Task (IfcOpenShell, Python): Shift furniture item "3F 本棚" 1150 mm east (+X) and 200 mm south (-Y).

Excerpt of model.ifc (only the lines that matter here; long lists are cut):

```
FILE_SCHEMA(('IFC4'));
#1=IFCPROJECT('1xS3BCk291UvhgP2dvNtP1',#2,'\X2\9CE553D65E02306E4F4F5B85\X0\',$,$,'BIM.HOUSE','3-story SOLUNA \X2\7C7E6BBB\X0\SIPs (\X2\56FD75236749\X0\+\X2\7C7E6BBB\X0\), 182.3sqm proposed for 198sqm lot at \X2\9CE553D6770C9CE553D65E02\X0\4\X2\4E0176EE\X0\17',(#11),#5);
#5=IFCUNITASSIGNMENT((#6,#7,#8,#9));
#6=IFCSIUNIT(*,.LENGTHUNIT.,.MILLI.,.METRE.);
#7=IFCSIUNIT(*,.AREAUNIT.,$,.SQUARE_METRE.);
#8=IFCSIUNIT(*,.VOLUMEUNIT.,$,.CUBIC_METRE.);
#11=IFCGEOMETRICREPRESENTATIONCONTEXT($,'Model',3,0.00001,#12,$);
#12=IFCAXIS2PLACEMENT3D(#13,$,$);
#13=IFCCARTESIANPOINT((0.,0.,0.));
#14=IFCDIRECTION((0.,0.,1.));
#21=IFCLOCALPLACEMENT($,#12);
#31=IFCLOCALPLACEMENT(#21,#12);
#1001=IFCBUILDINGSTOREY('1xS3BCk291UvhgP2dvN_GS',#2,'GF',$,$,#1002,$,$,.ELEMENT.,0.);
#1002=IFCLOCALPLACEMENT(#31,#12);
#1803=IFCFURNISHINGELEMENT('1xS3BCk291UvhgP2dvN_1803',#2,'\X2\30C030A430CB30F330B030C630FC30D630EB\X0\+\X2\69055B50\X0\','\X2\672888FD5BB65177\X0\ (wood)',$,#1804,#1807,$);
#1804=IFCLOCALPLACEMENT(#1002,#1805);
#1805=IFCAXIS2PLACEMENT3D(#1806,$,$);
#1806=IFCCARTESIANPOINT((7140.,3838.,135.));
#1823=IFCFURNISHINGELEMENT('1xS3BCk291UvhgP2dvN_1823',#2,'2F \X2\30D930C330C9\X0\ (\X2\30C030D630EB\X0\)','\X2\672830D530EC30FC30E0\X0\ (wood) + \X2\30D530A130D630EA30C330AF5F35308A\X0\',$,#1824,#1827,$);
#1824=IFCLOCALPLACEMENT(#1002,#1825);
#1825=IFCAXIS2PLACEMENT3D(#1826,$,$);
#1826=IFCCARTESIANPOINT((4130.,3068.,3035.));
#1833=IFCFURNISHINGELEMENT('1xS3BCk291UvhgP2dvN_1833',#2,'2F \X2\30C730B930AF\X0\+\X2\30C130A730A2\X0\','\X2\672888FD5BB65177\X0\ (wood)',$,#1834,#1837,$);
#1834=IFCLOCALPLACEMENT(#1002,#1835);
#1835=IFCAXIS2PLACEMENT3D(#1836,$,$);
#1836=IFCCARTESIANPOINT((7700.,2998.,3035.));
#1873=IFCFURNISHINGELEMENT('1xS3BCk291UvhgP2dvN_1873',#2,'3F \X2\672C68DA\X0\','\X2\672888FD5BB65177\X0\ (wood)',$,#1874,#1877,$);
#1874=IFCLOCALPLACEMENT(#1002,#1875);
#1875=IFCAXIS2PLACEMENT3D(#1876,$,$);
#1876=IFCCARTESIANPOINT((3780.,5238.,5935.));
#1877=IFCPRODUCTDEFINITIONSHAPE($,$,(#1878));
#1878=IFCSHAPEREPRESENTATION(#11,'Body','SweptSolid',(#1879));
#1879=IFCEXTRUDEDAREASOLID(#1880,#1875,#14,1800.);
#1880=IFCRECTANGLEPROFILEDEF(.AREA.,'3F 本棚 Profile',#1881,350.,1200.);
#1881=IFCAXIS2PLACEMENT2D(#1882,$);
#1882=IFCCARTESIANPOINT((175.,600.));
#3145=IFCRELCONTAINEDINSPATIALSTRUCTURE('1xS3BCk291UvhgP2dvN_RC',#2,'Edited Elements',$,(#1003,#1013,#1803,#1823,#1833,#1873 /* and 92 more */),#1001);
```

```python
import ifcopenshell
import ifcopenshell.api.geometry
import ifcopenshell.util.placement
import ifcopenshell.util.unit

model = ifcopenshell.open("model.ifc")
unit_scale = ifcopenshell.util.unit.calculate_unit_scale(model)

item = model.by_guid("1xS3BCk291UvhgP2dvN_1873")
matrix = ifcopenshell.util.placement.get_local_placement(item.ObjectPlacement)
matrix[0, 3] += 1.15 / unit_scale
matrix[1, 3] -= 0.2 / unit_scale
ifcopenshell.api.geometry.edit_object_placement(model, product=item, matrix=matrix, is_si=False)

print(ifcopenshell.util.placement.get_local_placement(item.ObjectPlacement).round(3) + 0.0)

model.write("model_rev.ifc")
```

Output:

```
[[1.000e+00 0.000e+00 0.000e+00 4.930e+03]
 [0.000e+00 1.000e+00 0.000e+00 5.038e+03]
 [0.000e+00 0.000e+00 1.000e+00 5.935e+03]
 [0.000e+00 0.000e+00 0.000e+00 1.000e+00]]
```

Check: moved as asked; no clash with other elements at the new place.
